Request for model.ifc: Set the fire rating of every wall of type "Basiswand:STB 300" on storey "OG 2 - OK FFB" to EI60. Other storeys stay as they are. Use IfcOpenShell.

First a look at what the model holds.

```python
import ifcopenshell
import ifcopenshell.util.element

model = ifcopenshell.open("model.ifc")
print(model.schema)
storey = next(s for s in model.by_type("IfcBuildingStorey") if s.Name == "OG 2 - OK FFB")
walls = [e for e in ifcopenshell.util.element.get_decomposition(storey) if e.is_a("IfcWall")]
seen = {}
for e in walls:
    element_type = ifcopenshell.util.element.get_type(e)
    key = (element_type.Name if element_type != e and element_type else None, ifcopenshell.util.element.get_pset(e, "Pset_WallCommon", "FireRating"))
    seen[key] = seen.get(key, 0) + 1
for (name, value), count in sorted(seen.items(), key=str):
    print(count, "x", name, "|", value)
```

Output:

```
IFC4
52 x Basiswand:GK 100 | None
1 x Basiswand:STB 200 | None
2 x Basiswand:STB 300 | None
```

```python
import ifcopenshell
import ifcopenshell.api.pset
import ifcopenshell.util.element

model = ifcopenshell.open("model.ifc")

storey = next(s for s in model.by_type("IfcBuildingStorey") if s.Name == "OG 2 - OK FFB")
walls = [e for e in ifcopenshell.util.element.get_decomposition(storey) if e.is_a("IfcWall")]

count = 0
for e in walls:
    element_type = ifcopenshell.util.element.get_type(e)
    if element_type in (None, e) or element_type.Name != "Basiswand:STB 300":
        continue
    # add_pset returns the element's existing set when there is one.
    pset = ifcopenshell.api.pset.add_pset(model, product=e, name="Pset_WallCommon")
    ifcopenshell.api.pset.edit_pset(model, pset=pset, properties={"FireRating": "EI60"})
    count += 1

print(count, "walls updated")

model.write("model_updated.ifc")
```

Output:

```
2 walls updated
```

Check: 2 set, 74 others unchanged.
